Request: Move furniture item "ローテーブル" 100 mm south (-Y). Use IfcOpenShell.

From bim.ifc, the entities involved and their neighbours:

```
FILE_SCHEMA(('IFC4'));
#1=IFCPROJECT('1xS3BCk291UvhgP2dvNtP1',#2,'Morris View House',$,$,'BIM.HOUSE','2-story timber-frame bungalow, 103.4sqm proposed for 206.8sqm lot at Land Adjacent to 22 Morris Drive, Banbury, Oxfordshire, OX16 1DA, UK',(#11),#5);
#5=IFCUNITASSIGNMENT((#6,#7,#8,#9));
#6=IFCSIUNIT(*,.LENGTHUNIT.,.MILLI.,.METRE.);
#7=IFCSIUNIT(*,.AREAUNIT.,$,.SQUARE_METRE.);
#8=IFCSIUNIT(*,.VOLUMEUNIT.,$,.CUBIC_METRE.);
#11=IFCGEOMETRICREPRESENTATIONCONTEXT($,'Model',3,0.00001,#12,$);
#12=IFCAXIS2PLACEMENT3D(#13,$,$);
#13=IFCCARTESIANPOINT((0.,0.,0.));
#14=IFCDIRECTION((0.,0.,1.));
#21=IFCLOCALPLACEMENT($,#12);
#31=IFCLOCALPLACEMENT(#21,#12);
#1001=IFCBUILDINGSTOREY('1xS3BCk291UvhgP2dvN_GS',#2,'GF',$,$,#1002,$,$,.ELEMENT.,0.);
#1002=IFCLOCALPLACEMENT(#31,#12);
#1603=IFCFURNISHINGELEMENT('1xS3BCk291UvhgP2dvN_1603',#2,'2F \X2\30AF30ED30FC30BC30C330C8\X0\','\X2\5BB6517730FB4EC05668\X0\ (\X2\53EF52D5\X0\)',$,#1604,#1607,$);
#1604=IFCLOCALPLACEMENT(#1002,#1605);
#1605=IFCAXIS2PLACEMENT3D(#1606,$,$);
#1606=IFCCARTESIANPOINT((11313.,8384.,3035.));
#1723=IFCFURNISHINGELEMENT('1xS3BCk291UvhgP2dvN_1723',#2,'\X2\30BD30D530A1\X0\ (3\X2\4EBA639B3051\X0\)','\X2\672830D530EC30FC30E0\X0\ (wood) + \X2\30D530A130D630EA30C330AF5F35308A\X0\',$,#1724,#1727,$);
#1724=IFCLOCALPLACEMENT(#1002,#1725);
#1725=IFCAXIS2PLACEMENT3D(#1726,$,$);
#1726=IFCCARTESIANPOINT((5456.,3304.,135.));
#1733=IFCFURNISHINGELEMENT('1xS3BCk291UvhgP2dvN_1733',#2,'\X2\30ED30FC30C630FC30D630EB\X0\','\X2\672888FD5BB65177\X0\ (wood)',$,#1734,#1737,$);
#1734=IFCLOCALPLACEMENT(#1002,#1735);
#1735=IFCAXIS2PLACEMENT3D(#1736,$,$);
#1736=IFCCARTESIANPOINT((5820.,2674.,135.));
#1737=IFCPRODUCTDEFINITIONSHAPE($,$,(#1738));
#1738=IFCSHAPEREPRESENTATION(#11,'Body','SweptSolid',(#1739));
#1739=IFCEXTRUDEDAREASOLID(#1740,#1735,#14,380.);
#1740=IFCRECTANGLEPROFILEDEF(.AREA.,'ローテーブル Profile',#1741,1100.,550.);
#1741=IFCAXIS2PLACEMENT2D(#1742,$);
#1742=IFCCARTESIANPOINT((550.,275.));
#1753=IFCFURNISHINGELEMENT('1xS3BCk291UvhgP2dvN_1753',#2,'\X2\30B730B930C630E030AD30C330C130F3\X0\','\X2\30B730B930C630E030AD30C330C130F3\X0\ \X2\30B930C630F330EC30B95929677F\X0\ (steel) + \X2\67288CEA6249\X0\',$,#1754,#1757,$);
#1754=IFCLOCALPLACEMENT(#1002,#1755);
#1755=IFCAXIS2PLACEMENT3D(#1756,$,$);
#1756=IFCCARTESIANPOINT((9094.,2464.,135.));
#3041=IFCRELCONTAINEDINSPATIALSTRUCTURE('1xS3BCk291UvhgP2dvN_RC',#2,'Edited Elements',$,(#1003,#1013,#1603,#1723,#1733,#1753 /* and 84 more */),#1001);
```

```python
import ifcopenshell
import ifcopenshell.api.geometry
import ifcopenshell.util.placement
import ifcopenshell.util.unit

model = ifcopenshell.open("bim.ifc")
unit_scale = ifcopenshell.util.unit.calculate_unit_scale(model)

item = model.by_guid("1xS3BCk291UvhgP2dvN_1733")
matrix = ifcopenshell.util.placement.get_local_placement(item.ObjectPlacement)
matrix[1, 3] -= 0.1 / unit_scale
ifcopenshell.api.geometry.edit_object_placement(model, product=item, matrix=matrix, is_si=False)

print(ifcopenshell.util.placement.get_local_placement(item.ObjectPlacement).round(3) + 0.0)

model.write("bim_edited.ifc")
```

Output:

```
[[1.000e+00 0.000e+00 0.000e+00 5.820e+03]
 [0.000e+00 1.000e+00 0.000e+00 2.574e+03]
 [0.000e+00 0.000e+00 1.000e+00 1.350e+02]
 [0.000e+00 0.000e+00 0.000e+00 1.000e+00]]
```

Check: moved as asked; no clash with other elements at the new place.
